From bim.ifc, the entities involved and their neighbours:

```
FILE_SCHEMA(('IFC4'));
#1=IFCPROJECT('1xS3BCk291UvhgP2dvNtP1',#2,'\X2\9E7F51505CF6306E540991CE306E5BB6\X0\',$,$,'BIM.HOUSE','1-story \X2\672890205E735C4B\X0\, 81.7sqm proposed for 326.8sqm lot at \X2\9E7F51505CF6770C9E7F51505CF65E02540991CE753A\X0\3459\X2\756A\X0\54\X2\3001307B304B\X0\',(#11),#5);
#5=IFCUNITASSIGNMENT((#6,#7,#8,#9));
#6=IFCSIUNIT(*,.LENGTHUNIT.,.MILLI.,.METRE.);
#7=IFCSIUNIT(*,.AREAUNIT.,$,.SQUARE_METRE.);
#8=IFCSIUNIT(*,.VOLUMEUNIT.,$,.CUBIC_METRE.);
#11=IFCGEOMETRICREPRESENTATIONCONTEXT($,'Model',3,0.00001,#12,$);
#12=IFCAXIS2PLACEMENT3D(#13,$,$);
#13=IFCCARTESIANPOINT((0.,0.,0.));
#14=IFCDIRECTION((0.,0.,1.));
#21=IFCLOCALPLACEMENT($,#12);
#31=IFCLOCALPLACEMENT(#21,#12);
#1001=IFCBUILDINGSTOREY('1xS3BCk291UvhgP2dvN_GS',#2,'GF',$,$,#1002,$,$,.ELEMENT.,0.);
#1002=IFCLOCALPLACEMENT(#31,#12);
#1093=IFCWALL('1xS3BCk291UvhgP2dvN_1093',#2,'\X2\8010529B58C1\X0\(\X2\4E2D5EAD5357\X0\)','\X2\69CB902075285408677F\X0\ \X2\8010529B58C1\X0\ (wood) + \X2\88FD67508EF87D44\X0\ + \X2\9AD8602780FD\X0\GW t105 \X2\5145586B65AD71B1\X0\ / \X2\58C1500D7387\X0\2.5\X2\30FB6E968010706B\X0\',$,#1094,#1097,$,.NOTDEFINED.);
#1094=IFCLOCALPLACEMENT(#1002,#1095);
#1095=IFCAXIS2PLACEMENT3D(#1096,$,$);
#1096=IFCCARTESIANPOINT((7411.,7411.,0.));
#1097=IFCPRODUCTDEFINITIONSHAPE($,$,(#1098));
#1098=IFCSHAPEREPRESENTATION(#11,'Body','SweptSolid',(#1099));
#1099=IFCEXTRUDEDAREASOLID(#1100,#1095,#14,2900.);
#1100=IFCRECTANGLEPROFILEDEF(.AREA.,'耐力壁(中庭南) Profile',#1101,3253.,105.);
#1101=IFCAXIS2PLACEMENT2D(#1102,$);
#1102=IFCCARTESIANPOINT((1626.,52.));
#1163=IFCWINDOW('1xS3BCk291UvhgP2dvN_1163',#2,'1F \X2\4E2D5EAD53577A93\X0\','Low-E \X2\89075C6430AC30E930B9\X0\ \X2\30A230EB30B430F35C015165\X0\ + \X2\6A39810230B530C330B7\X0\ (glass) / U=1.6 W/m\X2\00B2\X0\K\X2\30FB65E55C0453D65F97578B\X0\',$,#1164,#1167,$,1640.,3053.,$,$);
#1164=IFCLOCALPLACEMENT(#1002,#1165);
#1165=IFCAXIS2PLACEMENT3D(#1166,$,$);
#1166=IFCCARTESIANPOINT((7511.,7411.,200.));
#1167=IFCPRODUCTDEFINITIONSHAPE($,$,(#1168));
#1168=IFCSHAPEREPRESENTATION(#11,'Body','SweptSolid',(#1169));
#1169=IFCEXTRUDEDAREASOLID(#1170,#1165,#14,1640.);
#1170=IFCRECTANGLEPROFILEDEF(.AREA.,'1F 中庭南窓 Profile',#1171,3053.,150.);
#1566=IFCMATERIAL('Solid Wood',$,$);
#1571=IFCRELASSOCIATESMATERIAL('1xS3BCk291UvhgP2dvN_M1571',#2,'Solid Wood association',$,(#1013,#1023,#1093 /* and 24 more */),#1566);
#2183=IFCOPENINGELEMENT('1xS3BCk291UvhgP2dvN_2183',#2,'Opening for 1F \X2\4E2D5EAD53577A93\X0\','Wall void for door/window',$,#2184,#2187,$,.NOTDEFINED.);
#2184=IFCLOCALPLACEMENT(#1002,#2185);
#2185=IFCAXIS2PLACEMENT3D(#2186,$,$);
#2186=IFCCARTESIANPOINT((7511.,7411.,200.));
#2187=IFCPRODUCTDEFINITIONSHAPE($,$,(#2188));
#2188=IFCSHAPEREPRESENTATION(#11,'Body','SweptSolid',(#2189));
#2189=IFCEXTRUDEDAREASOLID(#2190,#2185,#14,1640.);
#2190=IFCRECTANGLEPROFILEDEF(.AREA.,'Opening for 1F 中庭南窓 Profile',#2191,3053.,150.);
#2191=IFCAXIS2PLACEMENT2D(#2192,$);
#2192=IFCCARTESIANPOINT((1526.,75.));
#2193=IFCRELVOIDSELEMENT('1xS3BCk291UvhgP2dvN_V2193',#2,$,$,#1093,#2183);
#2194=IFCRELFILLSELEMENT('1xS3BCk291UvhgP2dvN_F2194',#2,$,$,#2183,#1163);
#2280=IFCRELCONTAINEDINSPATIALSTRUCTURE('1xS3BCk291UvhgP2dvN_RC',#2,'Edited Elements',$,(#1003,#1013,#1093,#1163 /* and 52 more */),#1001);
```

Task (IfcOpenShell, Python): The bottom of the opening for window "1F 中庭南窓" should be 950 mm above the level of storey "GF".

```python
import numpy as np
import ifcopenshell
import ifcopenshell.api.geometry
import ifcopenshell.geom
import ifcopenshell.util.element
import ifcopenshell.util.placement
import ifcopenshell.util.shape
import ifcopenshell.util.unit

model = ifcopenshell.open("bim.ifc")
unit_scale = ifcopenshell.util.unit.calculate_unit_scale(model)

window = model.by_id(1163)
opening = window.FillsVoids[0].RelatingOpeningElement
storey = ifcopenshell.util.element.get_container(window, ifc_class="IfcBuildingStorey")
level = ifcopenshell.util.placement.get_local_placement(storey.ObjectPlacement)[2, 3]

# The opening's origin need not be at the sill, so measure its lowest point.
shape = ifcopenshell.geom.create_shape(ifcopenshell.geom.settings(), opening)
bottom = ifcopenshell.util.shape.get_shape_bottom_elevation(shape, shape.geometry) / unit_scale
dz = level + 0.95 / unit_scale - bottom

shift = np.array([0.0, 0.0, dz])
# The window is not placed relative to its opening, so move both.
for product in (opening, window):
    matrix = ifcopenshell.util.placement.get_local_placement(product.ObjectPlacement)
    matrix[:3, 3] += shift
    ifcopenshell.api.geometry.edit_object_placement(model, product=product, matrix=matrix, is_si=False)

print(f"moved by {dz * unit_scale:+.3f} m")

model.write("bim_v2.ifc")
```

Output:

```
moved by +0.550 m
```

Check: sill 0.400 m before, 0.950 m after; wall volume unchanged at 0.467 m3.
